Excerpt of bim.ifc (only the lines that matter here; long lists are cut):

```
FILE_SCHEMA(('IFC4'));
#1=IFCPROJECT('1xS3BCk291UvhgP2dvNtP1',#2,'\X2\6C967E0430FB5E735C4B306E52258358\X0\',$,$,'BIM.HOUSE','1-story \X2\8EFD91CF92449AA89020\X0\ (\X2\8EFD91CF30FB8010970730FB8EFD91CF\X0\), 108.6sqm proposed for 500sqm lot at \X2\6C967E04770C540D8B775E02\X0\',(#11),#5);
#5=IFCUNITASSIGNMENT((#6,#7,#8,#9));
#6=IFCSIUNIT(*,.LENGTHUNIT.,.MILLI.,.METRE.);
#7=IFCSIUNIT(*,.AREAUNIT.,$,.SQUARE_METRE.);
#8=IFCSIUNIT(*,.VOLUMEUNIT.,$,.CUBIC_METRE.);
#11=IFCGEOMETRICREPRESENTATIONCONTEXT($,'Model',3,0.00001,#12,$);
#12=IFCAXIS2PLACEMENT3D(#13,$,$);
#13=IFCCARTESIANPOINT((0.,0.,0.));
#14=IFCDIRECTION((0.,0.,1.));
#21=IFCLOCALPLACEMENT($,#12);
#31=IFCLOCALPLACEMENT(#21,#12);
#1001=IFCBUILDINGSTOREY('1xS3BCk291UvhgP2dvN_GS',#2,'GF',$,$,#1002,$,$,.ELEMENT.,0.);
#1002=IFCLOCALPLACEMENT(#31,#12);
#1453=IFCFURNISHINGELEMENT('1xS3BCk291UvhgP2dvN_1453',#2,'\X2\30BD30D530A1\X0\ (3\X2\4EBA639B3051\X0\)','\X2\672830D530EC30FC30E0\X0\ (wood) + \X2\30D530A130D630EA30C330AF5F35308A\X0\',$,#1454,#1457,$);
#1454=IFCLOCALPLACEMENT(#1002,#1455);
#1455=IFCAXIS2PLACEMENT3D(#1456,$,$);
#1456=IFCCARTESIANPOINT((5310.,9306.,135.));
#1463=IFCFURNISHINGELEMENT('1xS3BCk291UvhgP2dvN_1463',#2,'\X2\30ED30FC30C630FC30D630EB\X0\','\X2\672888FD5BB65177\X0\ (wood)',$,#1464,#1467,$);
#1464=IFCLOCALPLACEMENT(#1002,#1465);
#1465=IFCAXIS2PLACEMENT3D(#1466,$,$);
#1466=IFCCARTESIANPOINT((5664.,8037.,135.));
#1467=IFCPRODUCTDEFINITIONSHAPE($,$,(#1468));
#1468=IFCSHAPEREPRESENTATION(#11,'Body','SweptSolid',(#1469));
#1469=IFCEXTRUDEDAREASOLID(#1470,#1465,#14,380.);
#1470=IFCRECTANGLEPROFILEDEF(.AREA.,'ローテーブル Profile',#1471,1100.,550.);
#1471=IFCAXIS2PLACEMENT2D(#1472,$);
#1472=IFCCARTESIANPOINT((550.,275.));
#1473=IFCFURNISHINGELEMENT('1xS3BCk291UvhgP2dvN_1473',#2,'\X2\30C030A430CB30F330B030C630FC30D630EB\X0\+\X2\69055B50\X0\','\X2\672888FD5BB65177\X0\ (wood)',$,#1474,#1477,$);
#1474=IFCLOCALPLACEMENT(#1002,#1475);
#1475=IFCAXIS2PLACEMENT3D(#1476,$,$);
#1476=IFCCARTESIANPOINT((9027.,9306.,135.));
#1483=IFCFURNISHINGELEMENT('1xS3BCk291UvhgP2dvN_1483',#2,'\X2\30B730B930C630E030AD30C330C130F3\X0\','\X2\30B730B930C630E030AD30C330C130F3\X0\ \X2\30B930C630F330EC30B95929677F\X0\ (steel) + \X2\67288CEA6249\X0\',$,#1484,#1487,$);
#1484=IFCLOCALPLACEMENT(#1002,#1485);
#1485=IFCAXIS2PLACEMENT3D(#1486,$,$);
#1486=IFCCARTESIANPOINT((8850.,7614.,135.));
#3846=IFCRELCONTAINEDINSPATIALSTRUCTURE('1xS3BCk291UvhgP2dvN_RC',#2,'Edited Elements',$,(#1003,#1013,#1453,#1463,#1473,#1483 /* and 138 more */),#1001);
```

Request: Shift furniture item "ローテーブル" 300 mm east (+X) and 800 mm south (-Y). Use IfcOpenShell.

```python
import ifcopenshell
import ifcopenshell.api.geometry
import ifcopenshell.util.placement
import ifcopenshell.util.unit

model = ifcopenshell.open("bim.ifc")
unit_scale = ifcopenshell.util.unit.calculate_unit_scale(model)

item = model.by_id(1463)
matrix = ifcopenshell.util.placement.get_local_placement(item.ObjectPlacement)
matrix[0, 3] += 0.3 / unit_scale
matrix[1, 3] -= 0.8 / unit_scale
ifcopenshell.api.geometry.edit_object_placement(model, product=item, matrix=matrix, is_si=False)

print(ifcopenshell.util.placement.get_local_placement(item.ObjectPlacement).round(3) + 0.0)

model.write("bim_v2.ifc")
```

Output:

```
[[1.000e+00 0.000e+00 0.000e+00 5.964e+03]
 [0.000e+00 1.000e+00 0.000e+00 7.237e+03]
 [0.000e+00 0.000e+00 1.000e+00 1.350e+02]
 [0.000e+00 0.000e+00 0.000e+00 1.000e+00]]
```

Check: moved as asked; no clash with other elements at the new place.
